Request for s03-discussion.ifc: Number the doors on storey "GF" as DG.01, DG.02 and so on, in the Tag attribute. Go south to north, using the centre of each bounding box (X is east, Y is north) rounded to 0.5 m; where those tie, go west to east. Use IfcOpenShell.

First a look at what the model holds.

```python
import ifcopenshell
import ifcopenshell.util.element
import ifcopenshell.util.placement

model = ifcopenshell.open("s03-discussion.ifc")
print(model.schema)
storey = next(s for s in model.by_type("IfcBuildingStorey") if s.Name == "GF")
doors = [e for e in ifcopenshell.util.element.get_decomposition(storey) if e.is_a("IfcDoor")]
for e in sorted(doors, key=lambda e: e.id()):
    origin = ifcopenshell.util.placement.get_local_placement(e.ObjectPlacement)[:3, 3]
    print(e.id(), e.Tag, e.Name, origin.round(2) + 0.0, sep=" | ")
```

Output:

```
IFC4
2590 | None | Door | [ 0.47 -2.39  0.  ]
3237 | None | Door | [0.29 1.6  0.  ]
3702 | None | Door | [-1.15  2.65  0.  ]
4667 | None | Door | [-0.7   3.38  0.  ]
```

```python
import ifcopenshell
import ifcopenshell.geom
import ifcopenshell.util.element
import ifcopenshell.util.shape

model = ifcopenshell.open("s03-discussion.ifc")
settings = ifcopenshell.geom.settings()
settings.set("use-world-coords", True)


def centre(element):
    shape = ifcopenshell.geom.create_shape(settings, element)
    return ifcopenshell.util.shape.get_bbox_centroid(shape.geometry)


storey = next(s for s in model.by_type("IfcBuildingStorey") if s.Name == "GF")
doors = [e for e in ifcopenshell.util.element.get_decomposition(storey) if e.is_a("IfcDoor")]

# Insertion points can sit at a corner or the storey origin, so sort by the geometry (in metres).
centres = {e: centre(e) for e in doors}
doors.sort(key=lambda e: (round(centres[e][1] / 0.5), centres[e][0]))

for i, e in enumerate(doors, start=1):
    number = f"DG.{i:02d}"
    e.Tag = number
    print(e.id(), number)

model.write("s03-discussion_v2.ifc")
```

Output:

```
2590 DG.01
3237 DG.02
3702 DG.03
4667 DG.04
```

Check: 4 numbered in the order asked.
